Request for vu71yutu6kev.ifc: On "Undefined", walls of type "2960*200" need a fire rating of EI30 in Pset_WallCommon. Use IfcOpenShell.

First a look at what the model holds.

```python
import ifcopenshell
import ifcopenshell.util.element

model = ifcopenshell.open("vu71yutu6kev.ifc")
print(model.schema)
storey = next(s for s in model.by_type("IfcBuildingStorey") if s.Name == "Undefined")
walls = [e for e in ifcopenshell.util.element.get_decomposition(storey) if e.is_a("IfcWall")]
seen = {}
for e in walls:
    element_type = ifcopenshell.util.element.get_type(e)
    key = (element_type.Name if element_type != e and element_type else None, ifcopenshell.util.element.get_pset(e, "Pset_WallCommon", "FireRating"))
    seen[key] = seen.get(key, 0) + 1
for (name, value), count in sorted(seen.items(), key=str):
    print(count, "x", name, "|", value)
```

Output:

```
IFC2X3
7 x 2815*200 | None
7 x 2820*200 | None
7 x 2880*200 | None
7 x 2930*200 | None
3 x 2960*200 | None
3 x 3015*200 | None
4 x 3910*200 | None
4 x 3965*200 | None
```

```python
import ifcopenshell
import ifcopenshell.api.pset
import ifcopenshell.util.element

model = ifcopenshell.open("vu71yutu6kev.ifc")

storey = next(s for s in model.by_type("IfcBuildingStorey") if s.Name == "Undefined")
walls = [e for e in ifcopenshell.util.element.get_decomposition(storey) if e.is_a("IfcWall")]

count = 0
for e in walls:
    element_type = ifcopenshell.util.element.get_type(e)
    if element_type in (None, e) or element_type.Name != "2960*200":
        continue
    # add_pset returns the element's existing set when there is one.
    pset = ifcopenshell.api.pset.add_pset(model, product=e, name="Pset_WallCommon")
    ifcopenshell.api.pset.edit_pset(model, pset=pset, properties={"FireRating": "EI30"})
    count += 1

print(count, "walls updated")

model.write("vu71yutu6kev_edited.ifc")
```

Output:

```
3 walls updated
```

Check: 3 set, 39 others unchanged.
